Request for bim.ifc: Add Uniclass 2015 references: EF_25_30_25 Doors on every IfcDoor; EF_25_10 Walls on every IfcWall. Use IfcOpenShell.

First a look at what the model holds.

```python
import ifcopenshell

model = ifcopenshell.open("bim.ifc")
print(model.schema)
print("classifications:", [c.Name for c in model.by_type("IfcClassification")])
for ifc_class in ("IfcDoor", "IfcRoof", "IfcStair", "IfcWall", "IfcWindow"):
    print(ifc_class, len(model.by_type(ifc_class)))
```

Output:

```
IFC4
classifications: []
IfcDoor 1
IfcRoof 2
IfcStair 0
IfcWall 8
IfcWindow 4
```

```python
import ifcopenshell
import ifcopenshell.api.classification

model = ifcopenshell.open("bim.ifc")

system = ifcopenshell.api.classification.add_classification(model, classification="Uniclass 2015")

codes = {
    "IfcDoor": ("EF_25_30_25", "Doors"),
    "IfcWall": ("EF_25_10", "Walls"),
}
for ifc_class, (code, name) in codes.items():
    products = model.by_type(ifc_class)
    ifcopenshell.api.classification.add_reference(
        model, products=products, classification=system, identification=code, name=name
    )
    print(code, len(products))

model.write("bim-out.ifc")
```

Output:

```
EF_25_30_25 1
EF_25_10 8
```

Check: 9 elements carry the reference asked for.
